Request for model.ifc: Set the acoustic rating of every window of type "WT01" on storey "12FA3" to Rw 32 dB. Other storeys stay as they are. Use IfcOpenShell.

First a look at what the model holds.

```python
import ifcopenshell
import ifcopenshell.util.element

model = ifcopenshell.open("model.ifc")
print(model.schema)
storey = next(s for s in model.by_type("IfcBuildingStorey") if s.Name == "12FA3")
windows = [e for e in ifcopenshell.util.element.get_decomposition(storey) if e.is_a("IfcWindow")]
seen = {}
for e in windows:
    element_type = ifcopenshell.util.element.get_type(e)
    key = (element_type.Name if element_type != e and element_type else None, ifcopenshell.util.element.get_pset(e, "Pset_WindowCommon", "AcousticRating"))
    seen[key] = seen.get(key, 0) + 1
for (name, value), count in sorted(seen.items(), key=str):
    print(count, "x", name, "|", value)
```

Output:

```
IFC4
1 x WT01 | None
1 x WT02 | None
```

```python
import ifcopenshell
import ifcopenshell.api.pset
import ifcopenshell.util.element

model = ifcopenshell.open("model.ifc")

storey = next(s for s in model.by_type("IfcBuildingStorey") if s.Name == "12FA3")
windows = [e for e in ifcopenshell.util.element.get_decomposition(storey) if e.is_a("IfcWindow")]

count = 0
for e in windows:
    element_type = ifcopenshell.util.element.get_type(e)
    if element_type in (None, e) or element_type.Name != "WT01":
        continue
    # add_pset returns the element's existing set when there is one.
    pset = ifcopenshell.api.pset.add_pset(model, product=e, name="Pset_WindowCommon")
    ifcopenshell.api.pset.edit_pset(model, pset=pset, properties={"AcousticRating": "Rw 32 dB"})
    count += 1

print(count, "windows updated")

model.write("model_rev.ifc")
```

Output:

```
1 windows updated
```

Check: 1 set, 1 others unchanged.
